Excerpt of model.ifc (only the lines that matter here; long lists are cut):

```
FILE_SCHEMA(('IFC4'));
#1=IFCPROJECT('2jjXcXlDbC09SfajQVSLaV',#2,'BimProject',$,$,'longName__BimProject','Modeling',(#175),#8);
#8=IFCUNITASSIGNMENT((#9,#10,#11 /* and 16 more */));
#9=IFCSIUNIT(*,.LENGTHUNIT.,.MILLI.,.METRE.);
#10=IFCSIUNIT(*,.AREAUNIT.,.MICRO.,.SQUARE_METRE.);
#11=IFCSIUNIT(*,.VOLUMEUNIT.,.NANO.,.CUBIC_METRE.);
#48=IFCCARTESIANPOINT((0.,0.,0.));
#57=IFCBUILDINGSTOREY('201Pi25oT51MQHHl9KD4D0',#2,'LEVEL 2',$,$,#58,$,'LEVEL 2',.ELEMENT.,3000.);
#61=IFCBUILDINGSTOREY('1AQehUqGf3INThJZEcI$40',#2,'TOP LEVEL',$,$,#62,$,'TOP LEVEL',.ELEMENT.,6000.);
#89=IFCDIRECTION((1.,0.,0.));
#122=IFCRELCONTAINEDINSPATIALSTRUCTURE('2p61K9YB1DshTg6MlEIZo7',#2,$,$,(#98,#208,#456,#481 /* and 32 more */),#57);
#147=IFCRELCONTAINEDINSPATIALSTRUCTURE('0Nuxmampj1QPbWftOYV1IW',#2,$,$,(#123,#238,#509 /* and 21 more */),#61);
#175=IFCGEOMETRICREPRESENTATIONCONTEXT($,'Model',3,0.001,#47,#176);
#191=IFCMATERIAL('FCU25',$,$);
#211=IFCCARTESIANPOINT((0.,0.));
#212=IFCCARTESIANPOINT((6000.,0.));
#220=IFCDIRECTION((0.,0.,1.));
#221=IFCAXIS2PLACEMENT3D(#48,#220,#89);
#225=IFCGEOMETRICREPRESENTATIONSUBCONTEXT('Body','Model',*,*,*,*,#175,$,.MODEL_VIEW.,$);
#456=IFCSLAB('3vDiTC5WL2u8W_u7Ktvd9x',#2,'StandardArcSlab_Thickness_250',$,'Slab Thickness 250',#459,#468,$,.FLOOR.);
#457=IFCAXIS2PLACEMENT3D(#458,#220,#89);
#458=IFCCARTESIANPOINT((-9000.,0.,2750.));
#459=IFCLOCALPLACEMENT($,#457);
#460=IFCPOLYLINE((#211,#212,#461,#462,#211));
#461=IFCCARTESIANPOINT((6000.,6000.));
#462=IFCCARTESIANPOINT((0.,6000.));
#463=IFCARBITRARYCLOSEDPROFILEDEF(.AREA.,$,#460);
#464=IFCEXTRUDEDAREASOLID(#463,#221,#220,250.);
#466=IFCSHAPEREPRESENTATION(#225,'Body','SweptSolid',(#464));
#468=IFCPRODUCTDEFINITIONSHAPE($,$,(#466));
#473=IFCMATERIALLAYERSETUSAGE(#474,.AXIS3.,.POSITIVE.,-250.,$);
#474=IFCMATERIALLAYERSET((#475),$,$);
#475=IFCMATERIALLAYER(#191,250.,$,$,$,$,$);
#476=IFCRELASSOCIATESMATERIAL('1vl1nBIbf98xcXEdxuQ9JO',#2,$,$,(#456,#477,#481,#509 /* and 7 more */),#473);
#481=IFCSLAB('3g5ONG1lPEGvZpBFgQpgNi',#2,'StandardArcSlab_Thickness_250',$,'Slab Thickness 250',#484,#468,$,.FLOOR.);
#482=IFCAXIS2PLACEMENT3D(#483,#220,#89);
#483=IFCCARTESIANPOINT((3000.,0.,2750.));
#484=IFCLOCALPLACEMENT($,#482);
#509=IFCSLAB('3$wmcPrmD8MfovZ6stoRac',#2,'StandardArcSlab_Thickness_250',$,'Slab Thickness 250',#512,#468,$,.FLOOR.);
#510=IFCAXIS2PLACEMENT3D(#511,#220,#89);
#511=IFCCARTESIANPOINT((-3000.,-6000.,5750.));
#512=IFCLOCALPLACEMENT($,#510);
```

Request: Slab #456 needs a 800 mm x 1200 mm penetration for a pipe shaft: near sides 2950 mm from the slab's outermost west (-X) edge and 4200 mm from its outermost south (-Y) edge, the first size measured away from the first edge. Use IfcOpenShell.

```python
import numpy as np
import ifcopenshell
import ifcopenshell.api.feature
import ifcopenshell.api.geometry
import ifcopenshell.api.root
import ifcopenshell.geom
import ifcopenshell.util.placement
import ifcopenshell.util.representation
import ifcopenshell.util.shape
import ifcopenshell.util.unit

model = ifcopenshell.open("model.ifc")
unit_scale = ifcopenshell.util.unit.calculate_unit_scale(model)
settings = ifcopenshell.geom.settings()


def volume(element):
    """Net volume in cubic metres, openings subtracted."""
    shape = ifcopenshell.geom.create_shape(settings, element)
    return ifcopenshell.util.shape.get_volume(shape.geometry)


slab = model.by_id(456)
before = volume(slab)

# Extent in the slab's own axes, in metres. The edges named are its -X and -Y sides.
slab_shape = ifcopenshell.geom.create_shape(settings, slab)
vertices = ifcopenshell.util.shape.get_vertices(slab_shape.geometry)
x_min, y_min, bottom = vertices.min(axis=0)
top = vertices[:, 2].max()

opening = ifcopenshell.api.root.create_entity(model, ifc_class="IfcOpeningElement", name="Pipe shaft opening", predefined_type="OPENING")
context = ifcopenshell.util.representation.get_context(model, "Model", "Body", "MODEL_VIEW")
width, depth = 0.8, 1.2
outline = [(0.0, 0.0), (width, 0.0), (width, depth), (0.0, depth), (0.0, 0.0)]
# Overshoot both faces by 50 mm so the cut is clean.
shape = ifcopenshell.api.geometry.add_slab_representation(
    model, context=context, depth=top - bottom + 0.1, polyline=outline
)
ifcopenshell.api.geometry.assign_representation(model, product=opening, representation=shape)

matrix = ifcopenshell.util.placement.get_local_placement(slab.ObjectPlacement)
matrix[:, 3] = matrix @ np.append(np.array([x_min + 2.95, y_min + 4.2, bottom - 0.05]) / unit_scale, 1.0)
ifcopenshell.api.geometry.edit_object_placement(model, product=opening, matrix=matrix, is_si=False)
ifcopenshell.api.feature.add_feature(model, feature=opening, element=slab)

after = volume(slab)

print(f"slab volume {before:.3f} -> {after:.3f} m3")

model.write("model_rev.ifc")
```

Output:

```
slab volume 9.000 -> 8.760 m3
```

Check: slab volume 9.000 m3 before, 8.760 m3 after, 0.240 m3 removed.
